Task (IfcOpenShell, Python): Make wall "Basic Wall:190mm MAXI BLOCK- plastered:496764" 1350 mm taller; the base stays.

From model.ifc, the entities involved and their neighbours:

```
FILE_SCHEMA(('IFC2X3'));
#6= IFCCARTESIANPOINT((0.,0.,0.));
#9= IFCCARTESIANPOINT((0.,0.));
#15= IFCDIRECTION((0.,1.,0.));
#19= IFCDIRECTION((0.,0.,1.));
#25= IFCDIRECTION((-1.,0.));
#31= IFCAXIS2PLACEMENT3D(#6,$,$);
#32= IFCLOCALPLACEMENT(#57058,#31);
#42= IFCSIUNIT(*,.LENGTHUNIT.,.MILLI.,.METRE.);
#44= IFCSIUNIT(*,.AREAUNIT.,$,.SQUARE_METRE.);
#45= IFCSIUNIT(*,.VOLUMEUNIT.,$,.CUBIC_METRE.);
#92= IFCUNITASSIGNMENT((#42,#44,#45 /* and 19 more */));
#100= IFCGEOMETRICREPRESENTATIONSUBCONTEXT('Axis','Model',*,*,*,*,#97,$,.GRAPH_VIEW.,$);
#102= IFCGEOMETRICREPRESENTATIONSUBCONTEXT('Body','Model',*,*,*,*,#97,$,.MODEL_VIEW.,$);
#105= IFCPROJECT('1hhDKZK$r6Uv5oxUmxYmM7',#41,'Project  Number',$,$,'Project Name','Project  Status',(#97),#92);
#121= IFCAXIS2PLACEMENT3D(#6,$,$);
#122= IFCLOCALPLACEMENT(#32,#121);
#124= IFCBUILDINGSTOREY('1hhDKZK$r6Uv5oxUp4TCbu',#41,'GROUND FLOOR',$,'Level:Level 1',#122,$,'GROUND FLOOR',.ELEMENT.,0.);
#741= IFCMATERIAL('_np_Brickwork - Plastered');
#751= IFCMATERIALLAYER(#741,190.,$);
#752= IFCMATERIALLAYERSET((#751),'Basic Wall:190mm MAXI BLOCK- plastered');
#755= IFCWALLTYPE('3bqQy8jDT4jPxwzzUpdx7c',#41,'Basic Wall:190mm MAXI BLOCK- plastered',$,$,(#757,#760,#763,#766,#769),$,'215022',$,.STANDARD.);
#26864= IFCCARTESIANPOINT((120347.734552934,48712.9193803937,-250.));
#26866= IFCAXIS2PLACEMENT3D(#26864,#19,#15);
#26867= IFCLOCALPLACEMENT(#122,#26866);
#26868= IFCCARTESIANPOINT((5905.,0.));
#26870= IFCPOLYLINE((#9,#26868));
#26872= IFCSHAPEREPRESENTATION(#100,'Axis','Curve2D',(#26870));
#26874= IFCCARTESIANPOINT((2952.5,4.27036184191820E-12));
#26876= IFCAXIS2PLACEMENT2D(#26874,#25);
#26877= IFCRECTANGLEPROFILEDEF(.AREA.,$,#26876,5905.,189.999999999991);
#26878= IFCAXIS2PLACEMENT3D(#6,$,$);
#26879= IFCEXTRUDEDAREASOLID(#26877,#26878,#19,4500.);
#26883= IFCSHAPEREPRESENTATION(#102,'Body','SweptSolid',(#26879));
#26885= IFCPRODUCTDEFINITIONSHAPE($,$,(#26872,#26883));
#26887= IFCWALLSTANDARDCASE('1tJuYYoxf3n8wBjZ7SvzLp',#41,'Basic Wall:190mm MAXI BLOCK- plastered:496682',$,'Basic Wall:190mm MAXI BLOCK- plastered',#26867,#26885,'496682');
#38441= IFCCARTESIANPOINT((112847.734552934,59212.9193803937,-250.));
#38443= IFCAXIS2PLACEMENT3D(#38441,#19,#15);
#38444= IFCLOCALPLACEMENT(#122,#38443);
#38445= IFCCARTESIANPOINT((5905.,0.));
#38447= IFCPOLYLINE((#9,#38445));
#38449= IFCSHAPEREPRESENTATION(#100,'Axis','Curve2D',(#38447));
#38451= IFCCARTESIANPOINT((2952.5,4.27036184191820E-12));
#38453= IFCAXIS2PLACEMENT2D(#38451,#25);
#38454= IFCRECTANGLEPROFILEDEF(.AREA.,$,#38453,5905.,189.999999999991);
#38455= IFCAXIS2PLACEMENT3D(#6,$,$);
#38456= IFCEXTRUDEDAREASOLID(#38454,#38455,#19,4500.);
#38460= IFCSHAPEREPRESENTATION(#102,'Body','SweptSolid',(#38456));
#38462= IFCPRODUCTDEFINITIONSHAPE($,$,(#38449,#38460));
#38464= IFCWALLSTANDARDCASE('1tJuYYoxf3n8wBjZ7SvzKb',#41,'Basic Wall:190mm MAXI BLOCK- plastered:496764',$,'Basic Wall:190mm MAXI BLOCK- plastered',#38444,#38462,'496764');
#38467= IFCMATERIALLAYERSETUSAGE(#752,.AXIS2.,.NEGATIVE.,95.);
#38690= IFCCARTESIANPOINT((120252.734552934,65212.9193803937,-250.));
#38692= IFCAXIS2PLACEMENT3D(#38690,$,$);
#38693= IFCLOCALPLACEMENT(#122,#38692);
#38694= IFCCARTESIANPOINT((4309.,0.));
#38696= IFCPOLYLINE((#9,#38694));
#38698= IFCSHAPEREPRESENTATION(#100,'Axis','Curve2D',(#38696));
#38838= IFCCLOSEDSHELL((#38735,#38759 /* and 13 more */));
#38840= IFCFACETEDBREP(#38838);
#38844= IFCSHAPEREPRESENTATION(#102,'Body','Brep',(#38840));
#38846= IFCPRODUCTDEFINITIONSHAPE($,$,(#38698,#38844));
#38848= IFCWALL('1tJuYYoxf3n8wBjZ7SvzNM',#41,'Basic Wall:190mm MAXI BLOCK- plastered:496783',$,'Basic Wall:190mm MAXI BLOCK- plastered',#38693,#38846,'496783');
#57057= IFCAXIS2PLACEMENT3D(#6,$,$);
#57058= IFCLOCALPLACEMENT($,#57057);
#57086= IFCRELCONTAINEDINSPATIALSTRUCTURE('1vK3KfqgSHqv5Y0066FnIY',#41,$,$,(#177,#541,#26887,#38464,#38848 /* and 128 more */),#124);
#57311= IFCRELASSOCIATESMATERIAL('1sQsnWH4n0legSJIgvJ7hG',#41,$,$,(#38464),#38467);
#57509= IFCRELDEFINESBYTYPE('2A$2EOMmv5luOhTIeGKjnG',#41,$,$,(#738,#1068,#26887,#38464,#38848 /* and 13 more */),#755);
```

```python
import ifcopenshell
import ifcopenshell.geom
import ifcopenshell.util.representation
import ifcopenshell.util.shape

model = ifcopenshell.open("model.ifc")
settings = ifcopenshell.geom.settings()


def volume(element):
    """Net volume in cubic metres, openings subtracted."""
    shape = ifcopenshell.geom.create_shape(settings, element)
    return ifcopenshell.util.shape.get_volume(shape.geometry)


wall = model.by_guid("1tJuYYoxf3n8wBjZ7SvzKb")
before = volume(wall)

body = ifcopenshell.util.representation.get_representation(wall, "Model", "Body")
solid = body.Items[0]
old_height = solid.Depth
solid.Depth += 1350.0
after = volume(wall)

print(f"height {old_height:g} -> {solid.Depth:g}, volume {before:.3f} -> {after:.3f} m3")

model.write("model_edited.ifc")
```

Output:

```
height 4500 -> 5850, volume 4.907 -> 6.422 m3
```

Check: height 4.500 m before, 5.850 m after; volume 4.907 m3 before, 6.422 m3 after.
